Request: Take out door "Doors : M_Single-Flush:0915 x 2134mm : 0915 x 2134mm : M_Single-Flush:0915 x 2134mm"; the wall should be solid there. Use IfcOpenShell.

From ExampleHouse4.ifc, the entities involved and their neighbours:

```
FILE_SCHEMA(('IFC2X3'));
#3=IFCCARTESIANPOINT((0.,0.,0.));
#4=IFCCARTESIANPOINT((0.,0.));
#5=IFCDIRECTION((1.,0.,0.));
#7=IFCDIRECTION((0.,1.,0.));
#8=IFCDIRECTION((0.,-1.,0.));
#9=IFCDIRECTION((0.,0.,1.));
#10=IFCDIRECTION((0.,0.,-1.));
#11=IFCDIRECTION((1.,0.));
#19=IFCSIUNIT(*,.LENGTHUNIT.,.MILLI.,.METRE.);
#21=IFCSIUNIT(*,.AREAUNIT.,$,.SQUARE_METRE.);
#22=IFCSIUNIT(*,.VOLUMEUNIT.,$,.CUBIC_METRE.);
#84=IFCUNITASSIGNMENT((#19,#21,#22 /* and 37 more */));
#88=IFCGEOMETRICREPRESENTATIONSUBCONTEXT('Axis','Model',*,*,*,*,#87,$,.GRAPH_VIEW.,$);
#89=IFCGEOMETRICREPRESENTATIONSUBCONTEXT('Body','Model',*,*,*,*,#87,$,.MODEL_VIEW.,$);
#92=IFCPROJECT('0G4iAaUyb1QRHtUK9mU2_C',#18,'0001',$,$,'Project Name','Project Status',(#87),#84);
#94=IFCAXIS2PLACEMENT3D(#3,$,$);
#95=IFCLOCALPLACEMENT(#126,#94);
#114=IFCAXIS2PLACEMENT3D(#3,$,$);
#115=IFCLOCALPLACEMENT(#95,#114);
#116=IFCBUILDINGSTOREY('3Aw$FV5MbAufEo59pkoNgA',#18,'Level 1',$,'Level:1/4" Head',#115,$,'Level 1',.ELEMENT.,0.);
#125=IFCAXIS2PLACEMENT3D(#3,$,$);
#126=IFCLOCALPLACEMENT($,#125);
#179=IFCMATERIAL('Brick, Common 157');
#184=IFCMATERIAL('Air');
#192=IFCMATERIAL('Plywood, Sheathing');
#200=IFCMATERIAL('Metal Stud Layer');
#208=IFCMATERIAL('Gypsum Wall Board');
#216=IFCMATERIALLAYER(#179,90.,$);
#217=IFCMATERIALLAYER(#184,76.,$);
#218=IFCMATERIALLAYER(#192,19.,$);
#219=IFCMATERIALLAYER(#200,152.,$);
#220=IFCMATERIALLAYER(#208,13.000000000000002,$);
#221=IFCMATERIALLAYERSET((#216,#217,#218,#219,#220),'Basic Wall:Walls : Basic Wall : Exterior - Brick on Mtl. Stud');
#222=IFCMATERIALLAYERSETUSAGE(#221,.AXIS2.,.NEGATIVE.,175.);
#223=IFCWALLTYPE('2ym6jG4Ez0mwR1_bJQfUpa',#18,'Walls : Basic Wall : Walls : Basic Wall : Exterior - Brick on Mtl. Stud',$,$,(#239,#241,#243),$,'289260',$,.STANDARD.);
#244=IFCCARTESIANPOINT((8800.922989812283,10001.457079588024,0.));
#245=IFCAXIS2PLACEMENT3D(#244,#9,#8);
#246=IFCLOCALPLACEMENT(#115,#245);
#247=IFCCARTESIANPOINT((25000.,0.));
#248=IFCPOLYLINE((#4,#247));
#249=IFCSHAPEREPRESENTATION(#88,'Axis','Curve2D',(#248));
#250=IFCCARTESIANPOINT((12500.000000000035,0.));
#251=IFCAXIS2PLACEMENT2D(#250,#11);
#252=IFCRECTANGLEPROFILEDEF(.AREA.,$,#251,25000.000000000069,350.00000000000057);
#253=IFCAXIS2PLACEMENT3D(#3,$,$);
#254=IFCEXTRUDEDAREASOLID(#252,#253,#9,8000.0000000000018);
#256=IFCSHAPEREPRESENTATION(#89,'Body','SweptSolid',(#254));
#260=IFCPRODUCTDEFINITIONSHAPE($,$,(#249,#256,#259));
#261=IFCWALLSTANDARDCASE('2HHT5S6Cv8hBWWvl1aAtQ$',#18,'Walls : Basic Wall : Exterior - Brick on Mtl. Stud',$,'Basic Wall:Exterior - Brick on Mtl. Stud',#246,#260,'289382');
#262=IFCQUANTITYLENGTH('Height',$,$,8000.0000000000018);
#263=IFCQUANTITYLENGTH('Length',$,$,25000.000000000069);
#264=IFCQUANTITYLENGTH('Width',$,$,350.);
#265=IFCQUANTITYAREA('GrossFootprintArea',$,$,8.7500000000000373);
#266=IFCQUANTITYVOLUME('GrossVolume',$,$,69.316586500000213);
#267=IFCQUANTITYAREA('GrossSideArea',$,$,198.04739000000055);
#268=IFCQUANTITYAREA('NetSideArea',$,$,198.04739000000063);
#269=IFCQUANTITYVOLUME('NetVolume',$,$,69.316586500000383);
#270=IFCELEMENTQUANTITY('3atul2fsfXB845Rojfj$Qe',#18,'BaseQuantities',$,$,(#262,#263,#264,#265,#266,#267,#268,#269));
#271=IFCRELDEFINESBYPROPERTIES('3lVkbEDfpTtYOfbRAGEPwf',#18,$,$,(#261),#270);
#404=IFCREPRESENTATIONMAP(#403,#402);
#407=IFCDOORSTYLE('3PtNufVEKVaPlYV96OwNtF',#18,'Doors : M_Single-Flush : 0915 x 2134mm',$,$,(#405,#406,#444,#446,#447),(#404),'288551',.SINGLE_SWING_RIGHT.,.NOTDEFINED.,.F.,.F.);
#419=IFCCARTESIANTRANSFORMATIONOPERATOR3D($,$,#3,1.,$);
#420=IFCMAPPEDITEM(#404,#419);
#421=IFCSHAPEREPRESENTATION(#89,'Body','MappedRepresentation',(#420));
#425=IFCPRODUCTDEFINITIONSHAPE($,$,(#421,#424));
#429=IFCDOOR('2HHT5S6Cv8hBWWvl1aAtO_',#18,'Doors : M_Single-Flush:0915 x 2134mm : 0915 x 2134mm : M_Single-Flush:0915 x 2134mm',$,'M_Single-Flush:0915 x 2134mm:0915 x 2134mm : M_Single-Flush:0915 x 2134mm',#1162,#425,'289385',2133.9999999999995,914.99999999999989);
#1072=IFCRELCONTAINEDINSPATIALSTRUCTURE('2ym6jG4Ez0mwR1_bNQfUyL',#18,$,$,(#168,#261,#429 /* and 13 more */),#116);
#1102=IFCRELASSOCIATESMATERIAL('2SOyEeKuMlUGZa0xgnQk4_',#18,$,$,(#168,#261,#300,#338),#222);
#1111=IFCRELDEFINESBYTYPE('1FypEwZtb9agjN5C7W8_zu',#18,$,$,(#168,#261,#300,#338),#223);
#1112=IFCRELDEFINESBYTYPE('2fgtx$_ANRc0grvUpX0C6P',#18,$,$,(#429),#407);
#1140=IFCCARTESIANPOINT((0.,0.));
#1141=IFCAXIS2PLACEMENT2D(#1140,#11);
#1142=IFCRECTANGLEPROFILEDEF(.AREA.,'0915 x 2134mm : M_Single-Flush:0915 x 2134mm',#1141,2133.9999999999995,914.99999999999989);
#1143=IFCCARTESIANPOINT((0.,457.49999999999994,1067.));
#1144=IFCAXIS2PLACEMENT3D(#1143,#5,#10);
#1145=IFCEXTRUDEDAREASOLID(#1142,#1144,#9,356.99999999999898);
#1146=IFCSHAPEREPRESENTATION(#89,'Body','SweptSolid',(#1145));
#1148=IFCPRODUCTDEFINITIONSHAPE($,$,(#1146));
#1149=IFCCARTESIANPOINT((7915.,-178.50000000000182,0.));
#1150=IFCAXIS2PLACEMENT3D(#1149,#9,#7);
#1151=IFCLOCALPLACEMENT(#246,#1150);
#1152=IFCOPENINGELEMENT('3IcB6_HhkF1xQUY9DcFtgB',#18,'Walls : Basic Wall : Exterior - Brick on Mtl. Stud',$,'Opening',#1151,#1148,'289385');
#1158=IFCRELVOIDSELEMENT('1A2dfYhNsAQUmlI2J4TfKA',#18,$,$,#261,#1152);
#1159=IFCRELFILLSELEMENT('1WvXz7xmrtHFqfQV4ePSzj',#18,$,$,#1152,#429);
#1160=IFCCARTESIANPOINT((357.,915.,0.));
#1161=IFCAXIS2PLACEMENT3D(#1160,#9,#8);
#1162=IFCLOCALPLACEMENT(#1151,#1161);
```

```python
import ifcopenshell
import ifcopenshell.api.feature
import ifcopenshell.api.pset
import ifcopenshell.api.root
import ifcopenshell.geom
import ifcopenshell.util.element
import ifcopenshell.util.shape
import ifcopenshell.util.unit

model = ifcopenshell.open("ExampleHouse4.ifc")
area_scale = ifcopenshell.util.unit.calculate_unit_scale(model, "AREAUNIT")
volume_scale = ifcopenshell.util.unit.calculate_unit_scale(model, "VOLUMEUNIT")
settings = ifcopenshell.geom.settings()


def volume(element):
    """Net volume in cubic metres, openings subtracted."""
    shape = ifcopenshell.geom.create_shape(settings, element)
    return ifcopenshell.util.shape.get_volume(shape.geometry)


door = model.by_guid("2HHT5S6Cv8hBWWvl1aAtO_")
opening = door.FillsVoids[0].RelatingOpeningElement
wall = opening.VoidsElements[0].RelatingBuildingElement
before = volume(wall)

ifcopenshell.api.root.remove_product(model, product=door)
ifcopenshell.api.feature.remove_feature(model, feature=opening)

after = volume(wall)
thickness = 0.35  # wall thickness in metres

# Update the wall's stored quantities.
qto = model.by_id(ifcopenshell.util.element.get_pset(wall, "BaseQuantities", should_inherit=False)["id"])
ifcopenshell.api.pset.edit_qto(model, qto=qto, properties={
    "NetSideArea": after / thickness / area_scale,
    "NetVolume": after / volume_scale,
})

print(f"wall volume {before:.3f} -> {after:.3f} m3")

model.write("ExampleHouse4_updated.ifc")
```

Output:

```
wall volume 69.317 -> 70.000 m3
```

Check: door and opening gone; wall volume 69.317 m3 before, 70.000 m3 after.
